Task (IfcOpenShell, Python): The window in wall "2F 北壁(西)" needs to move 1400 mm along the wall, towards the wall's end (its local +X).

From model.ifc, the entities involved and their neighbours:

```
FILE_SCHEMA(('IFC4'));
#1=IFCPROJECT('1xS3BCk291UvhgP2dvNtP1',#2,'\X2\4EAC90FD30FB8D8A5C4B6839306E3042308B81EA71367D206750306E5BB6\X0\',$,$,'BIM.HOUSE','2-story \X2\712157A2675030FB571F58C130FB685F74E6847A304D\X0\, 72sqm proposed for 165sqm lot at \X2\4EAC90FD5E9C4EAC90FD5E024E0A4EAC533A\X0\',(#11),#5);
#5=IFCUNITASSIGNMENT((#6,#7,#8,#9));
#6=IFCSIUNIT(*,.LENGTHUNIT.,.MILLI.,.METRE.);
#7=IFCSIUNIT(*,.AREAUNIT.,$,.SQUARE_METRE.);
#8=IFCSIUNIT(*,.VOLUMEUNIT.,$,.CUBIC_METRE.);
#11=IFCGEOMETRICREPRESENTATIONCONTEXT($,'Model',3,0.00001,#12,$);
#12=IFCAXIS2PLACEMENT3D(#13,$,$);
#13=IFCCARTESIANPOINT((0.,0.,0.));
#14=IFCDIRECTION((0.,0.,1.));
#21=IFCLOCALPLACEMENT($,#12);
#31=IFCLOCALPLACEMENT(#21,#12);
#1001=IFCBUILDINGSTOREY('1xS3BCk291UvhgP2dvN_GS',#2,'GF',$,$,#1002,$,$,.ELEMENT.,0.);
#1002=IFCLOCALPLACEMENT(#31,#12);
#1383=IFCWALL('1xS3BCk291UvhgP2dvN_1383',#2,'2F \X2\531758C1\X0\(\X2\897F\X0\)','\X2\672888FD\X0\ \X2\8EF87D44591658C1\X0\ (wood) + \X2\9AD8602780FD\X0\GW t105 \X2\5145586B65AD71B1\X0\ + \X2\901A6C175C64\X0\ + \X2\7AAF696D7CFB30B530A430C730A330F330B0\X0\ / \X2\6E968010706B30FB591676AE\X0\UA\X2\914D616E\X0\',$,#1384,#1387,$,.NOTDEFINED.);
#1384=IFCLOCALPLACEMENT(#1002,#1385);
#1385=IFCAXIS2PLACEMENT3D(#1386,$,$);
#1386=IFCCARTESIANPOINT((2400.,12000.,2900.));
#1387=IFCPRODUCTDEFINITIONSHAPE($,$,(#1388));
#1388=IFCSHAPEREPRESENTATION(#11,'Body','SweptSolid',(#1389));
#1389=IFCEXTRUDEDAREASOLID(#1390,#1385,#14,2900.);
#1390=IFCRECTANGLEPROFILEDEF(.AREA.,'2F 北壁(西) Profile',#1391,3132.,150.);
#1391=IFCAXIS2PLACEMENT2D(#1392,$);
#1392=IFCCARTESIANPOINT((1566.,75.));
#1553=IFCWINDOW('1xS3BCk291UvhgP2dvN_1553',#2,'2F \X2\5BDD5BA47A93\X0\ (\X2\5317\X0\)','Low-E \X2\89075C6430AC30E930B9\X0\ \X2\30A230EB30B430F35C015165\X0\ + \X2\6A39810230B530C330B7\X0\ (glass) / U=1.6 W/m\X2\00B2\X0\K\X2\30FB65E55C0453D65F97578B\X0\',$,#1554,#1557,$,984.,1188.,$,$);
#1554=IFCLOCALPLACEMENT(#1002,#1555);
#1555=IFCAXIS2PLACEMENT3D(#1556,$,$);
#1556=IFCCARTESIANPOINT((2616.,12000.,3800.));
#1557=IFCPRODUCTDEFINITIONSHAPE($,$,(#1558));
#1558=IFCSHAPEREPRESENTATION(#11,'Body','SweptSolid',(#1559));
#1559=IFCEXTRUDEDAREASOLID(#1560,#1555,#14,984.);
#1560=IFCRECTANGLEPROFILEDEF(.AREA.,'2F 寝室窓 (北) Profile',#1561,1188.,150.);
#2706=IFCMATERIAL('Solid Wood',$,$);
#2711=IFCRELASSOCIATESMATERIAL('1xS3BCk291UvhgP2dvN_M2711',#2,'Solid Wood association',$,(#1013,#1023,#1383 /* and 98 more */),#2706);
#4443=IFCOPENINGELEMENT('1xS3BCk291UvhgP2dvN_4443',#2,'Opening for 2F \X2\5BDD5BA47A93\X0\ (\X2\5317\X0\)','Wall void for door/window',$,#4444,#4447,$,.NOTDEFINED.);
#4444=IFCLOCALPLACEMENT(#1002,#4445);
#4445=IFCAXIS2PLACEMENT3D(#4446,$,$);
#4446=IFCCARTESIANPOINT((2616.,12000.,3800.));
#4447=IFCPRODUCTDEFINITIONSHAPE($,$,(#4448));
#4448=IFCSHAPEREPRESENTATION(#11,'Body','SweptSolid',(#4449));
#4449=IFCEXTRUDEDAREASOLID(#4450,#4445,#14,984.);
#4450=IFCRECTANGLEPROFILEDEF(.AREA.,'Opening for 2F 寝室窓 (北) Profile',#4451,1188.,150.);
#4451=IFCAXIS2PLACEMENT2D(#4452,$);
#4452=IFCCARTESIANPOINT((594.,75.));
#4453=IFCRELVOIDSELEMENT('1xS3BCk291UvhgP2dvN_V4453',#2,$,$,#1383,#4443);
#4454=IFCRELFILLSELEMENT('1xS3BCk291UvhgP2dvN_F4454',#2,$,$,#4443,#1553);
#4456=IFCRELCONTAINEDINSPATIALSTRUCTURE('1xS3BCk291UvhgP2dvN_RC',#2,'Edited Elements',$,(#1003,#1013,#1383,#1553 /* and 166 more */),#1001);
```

```python
import ifcopenshell
import ifcopenshell.api.geometry
import ifcopenshell.util.placement
import ifcopenshell.util.unit

model = ifcopenshell.open("model.ifc")
unit_scale = ifcopenshell.util.unit.calculate_unit_scale(model)

window = model.by_guid("1xS3BCk291UvhgP2dvN_1553")
opening = window.FillsVoids[0].RelatingOpeningElement
wall = opening.VoidsElements[0].RelatingBuildingElement

wall_matrix = ifcopenshell.util.placement.get_local_placement(wall.ObjectPlacement)
shift = wall_matrix[:3, 0] * 1.4 / unit_scale
before = ifcopenshell.util.placement.get_local_placement(window.ObjectPlacement)[:3, 3].copy()

# The window is not placed relative to its opening, so move both.
for product in (opening, window):
    matrix = ifcopenshell.util.placement.get_local_placement(product.ObjectPlacement)
    matrix[:3, 3] += shift
    ifcopenshell.api.geometry.edit_object_placement(model, product=product, matrix=matrix, is_si=False)

after = ifcopenshell.util.placement.get_local_placement(window.ObjectPlacement)[:3, 3]
print("window moved by", (after - before).round(3) + 0.0)

model.write("model_updated.ifc")
```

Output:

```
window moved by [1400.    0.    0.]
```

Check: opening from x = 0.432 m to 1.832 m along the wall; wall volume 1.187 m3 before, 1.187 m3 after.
